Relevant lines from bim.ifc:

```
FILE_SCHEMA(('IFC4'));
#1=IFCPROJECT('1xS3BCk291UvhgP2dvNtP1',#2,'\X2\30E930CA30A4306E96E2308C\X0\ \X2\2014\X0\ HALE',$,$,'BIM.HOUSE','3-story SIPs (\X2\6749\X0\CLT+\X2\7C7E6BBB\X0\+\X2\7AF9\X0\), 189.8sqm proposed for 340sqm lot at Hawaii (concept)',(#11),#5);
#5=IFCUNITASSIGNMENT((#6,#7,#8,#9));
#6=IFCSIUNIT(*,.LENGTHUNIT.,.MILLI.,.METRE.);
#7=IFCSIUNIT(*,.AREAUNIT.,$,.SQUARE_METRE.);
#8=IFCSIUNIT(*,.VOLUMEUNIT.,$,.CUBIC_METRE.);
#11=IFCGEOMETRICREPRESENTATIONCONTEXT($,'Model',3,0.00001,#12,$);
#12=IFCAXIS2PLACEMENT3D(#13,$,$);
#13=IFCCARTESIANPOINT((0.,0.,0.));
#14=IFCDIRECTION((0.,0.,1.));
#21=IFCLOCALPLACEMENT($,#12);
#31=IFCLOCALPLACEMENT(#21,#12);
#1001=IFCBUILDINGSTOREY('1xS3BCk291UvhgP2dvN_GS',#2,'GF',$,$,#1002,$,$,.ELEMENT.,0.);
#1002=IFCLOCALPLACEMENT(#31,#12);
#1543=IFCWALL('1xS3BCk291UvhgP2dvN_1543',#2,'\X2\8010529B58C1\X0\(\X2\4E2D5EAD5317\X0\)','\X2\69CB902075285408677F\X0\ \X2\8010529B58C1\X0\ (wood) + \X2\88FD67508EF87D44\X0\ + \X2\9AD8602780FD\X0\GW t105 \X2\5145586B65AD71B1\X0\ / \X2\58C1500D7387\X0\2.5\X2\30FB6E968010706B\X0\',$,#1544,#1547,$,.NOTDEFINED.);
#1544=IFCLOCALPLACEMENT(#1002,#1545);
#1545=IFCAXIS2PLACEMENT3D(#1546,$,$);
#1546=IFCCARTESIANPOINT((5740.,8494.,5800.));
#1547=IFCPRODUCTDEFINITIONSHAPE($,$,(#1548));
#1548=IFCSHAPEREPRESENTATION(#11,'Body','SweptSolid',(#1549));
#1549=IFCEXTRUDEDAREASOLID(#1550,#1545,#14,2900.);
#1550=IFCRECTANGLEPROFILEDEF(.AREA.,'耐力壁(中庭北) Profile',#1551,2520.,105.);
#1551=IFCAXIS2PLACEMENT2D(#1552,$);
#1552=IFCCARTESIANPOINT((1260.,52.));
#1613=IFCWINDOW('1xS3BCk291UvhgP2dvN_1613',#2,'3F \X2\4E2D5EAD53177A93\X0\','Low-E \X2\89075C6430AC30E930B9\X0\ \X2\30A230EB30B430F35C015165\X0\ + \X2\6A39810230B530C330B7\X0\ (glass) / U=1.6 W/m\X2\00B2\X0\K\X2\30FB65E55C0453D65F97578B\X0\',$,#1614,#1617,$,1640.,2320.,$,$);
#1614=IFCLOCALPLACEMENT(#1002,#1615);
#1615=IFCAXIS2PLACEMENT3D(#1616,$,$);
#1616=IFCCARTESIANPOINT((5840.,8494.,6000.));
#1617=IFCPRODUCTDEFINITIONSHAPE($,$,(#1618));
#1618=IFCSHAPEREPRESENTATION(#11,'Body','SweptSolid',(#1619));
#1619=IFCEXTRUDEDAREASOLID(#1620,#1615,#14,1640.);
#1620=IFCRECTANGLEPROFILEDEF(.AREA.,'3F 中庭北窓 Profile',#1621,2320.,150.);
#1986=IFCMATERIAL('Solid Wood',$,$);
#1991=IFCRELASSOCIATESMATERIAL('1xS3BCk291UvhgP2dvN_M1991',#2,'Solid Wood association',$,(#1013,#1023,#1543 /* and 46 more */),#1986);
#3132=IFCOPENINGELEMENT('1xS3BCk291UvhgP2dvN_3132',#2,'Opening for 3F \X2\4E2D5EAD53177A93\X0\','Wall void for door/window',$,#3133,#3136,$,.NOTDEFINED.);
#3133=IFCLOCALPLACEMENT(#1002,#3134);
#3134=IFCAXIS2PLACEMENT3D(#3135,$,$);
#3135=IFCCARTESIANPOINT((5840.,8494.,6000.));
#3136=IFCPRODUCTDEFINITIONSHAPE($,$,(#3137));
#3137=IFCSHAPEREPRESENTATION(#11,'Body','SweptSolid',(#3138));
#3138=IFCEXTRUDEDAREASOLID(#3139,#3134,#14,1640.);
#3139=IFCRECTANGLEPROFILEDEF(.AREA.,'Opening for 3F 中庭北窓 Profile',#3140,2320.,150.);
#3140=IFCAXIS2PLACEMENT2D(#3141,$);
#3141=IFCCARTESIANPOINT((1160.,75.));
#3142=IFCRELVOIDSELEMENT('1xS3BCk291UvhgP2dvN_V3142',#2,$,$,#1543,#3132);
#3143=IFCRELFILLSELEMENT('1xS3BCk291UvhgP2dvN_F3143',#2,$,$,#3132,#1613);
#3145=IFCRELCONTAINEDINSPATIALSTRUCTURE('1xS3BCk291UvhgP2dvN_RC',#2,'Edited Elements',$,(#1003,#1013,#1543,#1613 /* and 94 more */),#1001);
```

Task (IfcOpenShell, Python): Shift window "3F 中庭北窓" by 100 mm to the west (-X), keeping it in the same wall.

```python
import ifcopenshell
import ifcopenshell.api.geometry
import ifcopenshell.util.placement

model = ifcopenshell.open("bim.ifc")

window = model.by_guid("1xS3BCk291UvhgP2dvN_1613")
opening = window.FillsVoids[0].RelatingOpeningElement
wall = opening.VoidsElements[0].RelatingBuildingElement

wall_matrix = ifcopenshell.util.placement.get_local_placement(wall.ObjectPlacement)
shift = wall_matrix[:3, 0] * -100.0
before = ifcopenshell.util.placement.get_local_placement(window.ObjectPlacement)[:3, 3].copy()

# The window is not placed relative to its opening, so move both.
for product in (opening, window):
    matrix = ifcopenshell.util.placement.get_local_placement(product.ObjectPlacement)
    matrix[:3, 3] += shift
    ifcopenshell.api.geometry.edit_object_placement(model, product=product, matrix=matrix, is_si=False)

after = ifcopenshell.util.placement.get_local_placement(window.ObjectPlacement)[:3, 3]
print("window moved by", (after - before).round(3) + 0.0)

model.write("bim_v2.ifc")
```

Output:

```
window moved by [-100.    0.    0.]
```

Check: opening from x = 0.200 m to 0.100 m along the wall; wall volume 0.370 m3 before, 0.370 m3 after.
